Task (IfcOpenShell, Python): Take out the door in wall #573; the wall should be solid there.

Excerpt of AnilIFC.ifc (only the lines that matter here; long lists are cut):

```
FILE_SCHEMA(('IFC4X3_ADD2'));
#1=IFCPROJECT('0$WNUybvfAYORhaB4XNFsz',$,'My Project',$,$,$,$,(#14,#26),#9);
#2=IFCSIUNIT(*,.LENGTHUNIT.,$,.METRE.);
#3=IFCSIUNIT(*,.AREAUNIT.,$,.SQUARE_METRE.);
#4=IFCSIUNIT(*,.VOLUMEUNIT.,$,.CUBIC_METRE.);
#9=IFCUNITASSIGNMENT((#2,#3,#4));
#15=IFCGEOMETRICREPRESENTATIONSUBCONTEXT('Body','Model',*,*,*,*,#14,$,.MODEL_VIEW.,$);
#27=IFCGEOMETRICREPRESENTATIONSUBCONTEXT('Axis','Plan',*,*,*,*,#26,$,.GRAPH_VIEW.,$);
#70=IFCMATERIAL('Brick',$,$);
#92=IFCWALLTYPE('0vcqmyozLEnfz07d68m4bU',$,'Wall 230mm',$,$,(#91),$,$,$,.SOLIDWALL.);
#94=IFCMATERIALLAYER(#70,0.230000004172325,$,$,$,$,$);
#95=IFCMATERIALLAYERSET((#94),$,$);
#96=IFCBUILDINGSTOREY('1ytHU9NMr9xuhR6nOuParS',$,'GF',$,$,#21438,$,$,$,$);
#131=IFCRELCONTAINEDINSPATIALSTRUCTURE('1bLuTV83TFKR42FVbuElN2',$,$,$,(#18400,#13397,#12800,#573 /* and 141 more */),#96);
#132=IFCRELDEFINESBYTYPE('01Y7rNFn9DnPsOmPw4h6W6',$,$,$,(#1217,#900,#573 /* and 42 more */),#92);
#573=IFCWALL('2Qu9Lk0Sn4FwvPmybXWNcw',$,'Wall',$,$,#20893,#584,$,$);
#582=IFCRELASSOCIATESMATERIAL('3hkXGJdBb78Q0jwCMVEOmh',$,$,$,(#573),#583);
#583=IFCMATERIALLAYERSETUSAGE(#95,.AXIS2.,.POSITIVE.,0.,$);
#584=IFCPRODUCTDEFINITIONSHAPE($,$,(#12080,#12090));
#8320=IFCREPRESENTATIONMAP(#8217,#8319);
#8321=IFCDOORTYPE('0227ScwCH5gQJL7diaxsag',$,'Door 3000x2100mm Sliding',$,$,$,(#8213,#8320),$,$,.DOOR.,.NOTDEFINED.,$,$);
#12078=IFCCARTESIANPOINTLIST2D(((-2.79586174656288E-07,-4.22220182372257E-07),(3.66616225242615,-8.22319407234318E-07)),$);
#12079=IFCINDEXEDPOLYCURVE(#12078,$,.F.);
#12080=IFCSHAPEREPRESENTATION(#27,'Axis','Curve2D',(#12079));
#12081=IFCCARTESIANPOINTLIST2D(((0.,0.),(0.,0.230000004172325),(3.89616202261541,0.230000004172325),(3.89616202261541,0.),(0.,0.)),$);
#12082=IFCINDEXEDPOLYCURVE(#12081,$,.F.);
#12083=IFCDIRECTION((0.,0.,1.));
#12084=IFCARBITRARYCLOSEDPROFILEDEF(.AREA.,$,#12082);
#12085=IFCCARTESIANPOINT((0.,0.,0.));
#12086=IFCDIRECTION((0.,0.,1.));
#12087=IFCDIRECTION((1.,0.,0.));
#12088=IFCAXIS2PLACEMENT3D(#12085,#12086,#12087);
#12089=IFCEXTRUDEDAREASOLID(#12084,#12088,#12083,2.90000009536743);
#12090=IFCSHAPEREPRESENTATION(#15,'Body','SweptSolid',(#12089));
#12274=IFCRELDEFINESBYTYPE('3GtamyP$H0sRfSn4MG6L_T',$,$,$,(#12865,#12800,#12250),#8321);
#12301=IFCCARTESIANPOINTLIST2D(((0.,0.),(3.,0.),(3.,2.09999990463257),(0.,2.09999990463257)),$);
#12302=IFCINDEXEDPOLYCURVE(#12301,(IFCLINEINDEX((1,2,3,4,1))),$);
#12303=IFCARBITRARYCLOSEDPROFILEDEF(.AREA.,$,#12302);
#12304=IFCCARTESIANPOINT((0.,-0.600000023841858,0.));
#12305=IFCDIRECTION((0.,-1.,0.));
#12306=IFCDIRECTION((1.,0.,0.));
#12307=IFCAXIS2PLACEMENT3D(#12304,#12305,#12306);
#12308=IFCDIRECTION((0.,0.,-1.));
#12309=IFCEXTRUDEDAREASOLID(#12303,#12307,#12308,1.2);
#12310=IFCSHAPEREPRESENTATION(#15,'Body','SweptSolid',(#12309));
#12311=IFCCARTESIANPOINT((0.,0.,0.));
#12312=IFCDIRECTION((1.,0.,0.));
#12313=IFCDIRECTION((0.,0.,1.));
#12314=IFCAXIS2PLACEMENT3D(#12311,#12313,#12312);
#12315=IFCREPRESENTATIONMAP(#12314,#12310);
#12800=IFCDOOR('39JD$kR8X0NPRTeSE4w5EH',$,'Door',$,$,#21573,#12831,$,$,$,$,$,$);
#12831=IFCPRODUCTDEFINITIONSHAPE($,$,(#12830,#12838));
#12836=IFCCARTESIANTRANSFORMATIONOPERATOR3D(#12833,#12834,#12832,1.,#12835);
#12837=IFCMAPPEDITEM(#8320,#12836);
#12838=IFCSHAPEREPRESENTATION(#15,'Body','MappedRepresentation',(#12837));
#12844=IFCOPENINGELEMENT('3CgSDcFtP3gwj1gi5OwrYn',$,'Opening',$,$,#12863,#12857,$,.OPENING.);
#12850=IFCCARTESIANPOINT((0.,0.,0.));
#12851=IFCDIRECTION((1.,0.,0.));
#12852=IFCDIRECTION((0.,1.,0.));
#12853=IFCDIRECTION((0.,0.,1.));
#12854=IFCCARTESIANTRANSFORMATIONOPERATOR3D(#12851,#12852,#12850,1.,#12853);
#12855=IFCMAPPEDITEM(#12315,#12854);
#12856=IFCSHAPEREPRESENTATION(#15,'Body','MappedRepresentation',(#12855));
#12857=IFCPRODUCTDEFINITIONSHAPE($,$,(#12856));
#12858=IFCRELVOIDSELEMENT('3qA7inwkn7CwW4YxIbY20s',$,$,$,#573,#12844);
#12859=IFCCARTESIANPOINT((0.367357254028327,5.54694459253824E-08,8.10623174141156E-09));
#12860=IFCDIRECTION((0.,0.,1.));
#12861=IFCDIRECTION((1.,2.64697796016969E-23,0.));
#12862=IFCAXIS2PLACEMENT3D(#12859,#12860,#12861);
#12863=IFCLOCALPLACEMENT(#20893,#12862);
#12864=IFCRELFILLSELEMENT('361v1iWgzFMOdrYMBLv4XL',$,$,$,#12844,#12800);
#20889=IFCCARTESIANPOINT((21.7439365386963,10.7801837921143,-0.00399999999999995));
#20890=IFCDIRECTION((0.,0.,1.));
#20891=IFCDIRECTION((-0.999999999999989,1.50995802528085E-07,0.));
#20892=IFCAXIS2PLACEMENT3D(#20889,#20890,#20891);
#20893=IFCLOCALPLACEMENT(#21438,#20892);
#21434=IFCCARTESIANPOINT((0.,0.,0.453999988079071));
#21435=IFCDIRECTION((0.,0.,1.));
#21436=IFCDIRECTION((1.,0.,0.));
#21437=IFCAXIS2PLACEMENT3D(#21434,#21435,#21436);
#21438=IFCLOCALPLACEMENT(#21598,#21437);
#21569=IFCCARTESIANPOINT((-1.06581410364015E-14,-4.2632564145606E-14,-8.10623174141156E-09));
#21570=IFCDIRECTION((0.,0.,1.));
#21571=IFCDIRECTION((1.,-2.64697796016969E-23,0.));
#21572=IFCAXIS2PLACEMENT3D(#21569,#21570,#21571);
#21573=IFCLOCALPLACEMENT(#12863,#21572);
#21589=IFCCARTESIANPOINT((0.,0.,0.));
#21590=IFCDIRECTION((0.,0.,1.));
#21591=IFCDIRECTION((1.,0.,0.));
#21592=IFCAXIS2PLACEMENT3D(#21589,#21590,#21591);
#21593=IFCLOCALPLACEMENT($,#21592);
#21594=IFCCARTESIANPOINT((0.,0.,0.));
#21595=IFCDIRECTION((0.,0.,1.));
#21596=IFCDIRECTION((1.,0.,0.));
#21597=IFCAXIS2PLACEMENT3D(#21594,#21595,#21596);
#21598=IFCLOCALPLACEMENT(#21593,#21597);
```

```python
import ifcopenshell
import ifcopenshell.api.feature
import ifcopenshell.api.root
import ifcopenshell.geom
import ifcopenshell.util.shape

model = ifcopenshell.open("AnilIFC.ifc")
settings = ifcopenshell.geom.settings()


def volume(element):
    """Net volume in cubic metres, openings subtracted."""
    shape = ifcopenshell.geom.create_shape(settings, element)
    return ifcopenshell.util.shape.get_volume(shape.geometry)


door = model.by_guid("39JD$kR8X0NPRTeSE4w5EH")
opening = door.FillsVoids[0].RelatingOpeningElement
wall = opening.VoidsElements[0].RelatingBuildingElement
before = volume(wall)

ifcopenshell.api.root.remove_product(model, product=door)
ifcopenshell.api.feature.remove_feature(model, feature=opening)

after = volume(wall)

print(f"wall volume {before:.3f} -> {after:.3f} m3")

model.write("AnilIFC_edited.ifc")
```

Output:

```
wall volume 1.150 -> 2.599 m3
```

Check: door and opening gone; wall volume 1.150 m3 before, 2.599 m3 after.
